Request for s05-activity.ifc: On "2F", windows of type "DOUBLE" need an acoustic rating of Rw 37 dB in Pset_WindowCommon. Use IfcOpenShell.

First a look at what the model holds.

```python
import ifcopenshell
import ifcopenshell.util.element

model = ifcopenshell.open("s05-activity.ifc")
print(model.schema)
storey = next(s for s in model.by_type("IfcBuildingStorey") if s.Name == "2F")
windows = [e for e in ifcopenshell.util.element.get_decomposition(storey) if e.is_a("IfcWindow")]
seen = {}
for e in windows:
    element_type = ifcopenshell.util.element.get_type(e)
    key = (element_type.Name if element_type != e and element_type else None, ifcopenshell.util.element.get_pset(e, "Pset_WindowCommon", "AcousticRating"))
    seen[key] = seen.get(key, 0) + 1
for (name, value), count in sorted(seen.items(), key=str):
    print(count, "x", name, "|", value)
```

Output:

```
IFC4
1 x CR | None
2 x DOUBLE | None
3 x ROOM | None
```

```python
import ifcopenshell
import ifcopenshell.api.pset
import ifcopenshell.util.element

model = ifcopenshell.open("s05-activity.ifc")

storey = next(s for s in model.by_type("IfcBuildingStorey") if s.Name == "2F")
windows = [e for e in ifcopenshell.util.element.get_decomposition(storey) if e.is_a("IfcWindow")]

count = 0
for e in windows:
    element_type = ifcopenshell.util.element.get_type(e)
    if element_type in (None, e) or element_type.Name != "DOUBLE":
        continue
    # add_pset returns the element's existing set when there is one.
    pset = ifcopenshell.api.pset.add_pset(model, product=e, name="Pset_WindowCommon")
    ifcopenshell.api.pset.edit_pset(model, pset=pset, properties={"AcousticRating": "Rw 37 dB"})
    count += 1

print(count, "windows updated")

model.write("s05-activity_updated.ifc")
```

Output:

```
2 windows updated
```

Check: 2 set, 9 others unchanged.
